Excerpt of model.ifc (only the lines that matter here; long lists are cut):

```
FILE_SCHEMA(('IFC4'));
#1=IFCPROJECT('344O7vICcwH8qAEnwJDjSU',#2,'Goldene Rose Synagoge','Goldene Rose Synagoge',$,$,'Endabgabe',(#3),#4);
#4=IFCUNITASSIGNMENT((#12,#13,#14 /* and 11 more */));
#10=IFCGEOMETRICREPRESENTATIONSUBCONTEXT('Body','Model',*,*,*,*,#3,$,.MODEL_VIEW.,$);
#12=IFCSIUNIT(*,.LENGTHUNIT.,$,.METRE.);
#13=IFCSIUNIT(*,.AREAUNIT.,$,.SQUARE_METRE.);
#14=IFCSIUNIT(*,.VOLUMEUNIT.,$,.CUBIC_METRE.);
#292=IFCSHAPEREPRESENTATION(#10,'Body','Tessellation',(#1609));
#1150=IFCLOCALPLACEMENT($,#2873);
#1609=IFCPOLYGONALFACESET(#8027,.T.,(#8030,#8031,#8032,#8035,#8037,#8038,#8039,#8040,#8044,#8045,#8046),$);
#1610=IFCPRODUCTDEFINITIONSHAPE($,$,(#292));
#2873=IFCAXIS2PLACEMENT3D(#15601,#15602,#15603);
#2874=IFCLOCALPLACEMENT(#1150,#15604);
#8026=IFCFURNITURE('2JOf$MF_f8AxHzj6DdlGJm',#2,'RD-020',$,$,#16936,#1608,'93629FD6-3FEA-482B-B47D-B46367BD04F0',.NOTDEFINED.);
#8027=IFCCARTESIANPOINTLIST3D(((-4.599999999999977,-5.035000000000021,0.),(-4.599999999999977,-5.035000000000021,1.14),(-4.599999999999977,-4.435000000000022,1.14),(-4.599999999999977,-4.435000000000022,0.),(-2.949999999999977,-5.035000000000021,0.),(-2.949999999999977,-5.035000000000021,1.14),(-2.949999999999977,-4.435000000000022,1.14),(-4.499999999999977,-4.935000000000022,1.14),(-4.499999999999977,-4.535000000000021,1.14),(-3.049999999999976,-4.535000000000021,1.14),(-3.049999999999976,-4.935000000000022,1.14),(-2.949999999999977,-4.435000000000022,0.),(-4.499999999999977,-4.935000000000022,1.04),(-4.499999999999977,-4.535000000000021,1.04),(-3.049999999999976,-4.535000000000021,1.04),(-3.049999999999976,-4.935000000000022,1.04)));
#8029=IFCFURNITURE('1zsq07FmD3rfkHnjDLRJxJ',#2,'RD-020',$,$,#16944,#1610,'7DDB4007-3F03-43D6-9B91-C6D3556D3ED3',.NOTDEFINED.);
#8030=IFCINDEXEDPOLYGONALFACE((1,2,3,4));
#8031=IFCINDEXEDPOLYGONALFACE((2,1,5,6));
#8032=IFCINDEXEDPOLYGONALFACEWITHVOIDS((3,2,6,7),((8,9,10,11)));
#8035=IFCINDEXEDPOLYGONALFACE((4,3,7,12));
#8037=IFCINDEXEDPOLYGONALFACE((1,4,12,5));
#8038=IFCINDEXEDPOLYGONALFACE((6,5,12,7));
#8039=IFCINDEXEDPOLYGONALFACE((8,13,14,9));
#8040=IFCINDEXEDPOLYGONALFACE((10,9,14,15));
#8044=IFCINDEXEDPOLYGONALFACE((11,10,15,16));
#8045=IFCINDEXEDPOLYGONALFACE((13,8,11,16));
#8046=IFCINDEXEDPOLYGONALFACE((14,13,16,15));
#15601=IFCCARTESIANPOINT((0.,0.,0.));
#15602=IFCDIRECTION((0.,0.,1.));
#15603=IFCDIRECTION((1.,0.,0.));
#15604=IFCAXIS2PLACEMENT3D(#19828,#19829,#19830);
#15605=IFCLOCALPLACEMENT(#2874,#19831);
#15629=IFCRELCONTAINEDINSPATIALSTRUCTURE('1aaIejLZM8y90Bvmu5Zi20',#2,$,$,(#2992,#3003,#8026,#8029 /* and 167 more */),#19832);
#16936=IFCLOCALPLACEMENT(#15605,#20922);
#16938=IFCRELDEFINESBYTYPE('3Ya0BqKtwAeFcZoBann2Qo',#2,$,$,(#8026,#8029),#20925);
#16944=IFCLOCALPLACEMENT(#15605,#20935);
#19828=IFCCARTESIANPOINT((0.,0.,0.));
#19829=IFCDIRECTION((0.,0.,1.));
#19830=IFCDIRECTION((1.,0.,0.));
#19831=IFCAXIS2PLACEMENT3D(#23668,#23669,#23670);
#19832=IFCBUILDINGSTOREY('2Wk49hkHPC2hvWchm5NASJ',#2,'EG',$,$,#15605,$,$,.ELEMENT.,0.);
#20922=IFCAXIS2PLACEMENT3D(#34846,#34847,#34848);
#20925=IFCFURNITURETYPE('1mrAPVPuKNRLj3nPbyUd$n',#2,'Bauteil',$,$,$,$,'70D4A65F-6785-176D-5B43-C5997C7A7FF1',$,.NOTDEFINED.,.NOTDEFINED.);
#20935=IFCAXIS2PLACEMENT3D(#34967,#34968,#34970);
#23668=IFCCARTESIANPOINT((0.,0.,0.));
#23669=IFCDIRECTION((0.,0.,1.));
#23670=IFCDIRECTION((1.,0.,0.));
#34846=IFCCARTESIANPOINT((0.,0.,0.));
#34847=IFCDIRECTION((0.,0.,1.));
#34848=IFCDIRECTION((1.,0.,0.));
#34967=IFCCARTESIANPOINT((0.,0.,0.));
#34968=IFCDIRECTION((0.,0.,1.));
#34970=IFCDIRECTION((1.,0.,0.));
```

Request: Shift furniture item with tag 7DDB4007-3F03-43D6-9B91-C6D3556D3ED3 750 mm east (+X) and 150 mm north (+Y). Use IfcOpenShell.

```python
import ifcopenshell
import ifcopenshell.api.geometry
import ifcopenshell.util.placement
import ifcopenshell.util.unit

model = ifcopenshell.open("model.ifc")
unit_scale = ifcopenshell.util.unit.calculate_unit_scale(model)

item = model.by_id(8029)
matrix = ifcopenshell.util.placement.get_local_placement(item.ObjectPlacement)
matrix[0, 3] += 0.75 / unit_scale
matrix[1, 3] += 0.15 / unit_scale
ifcopenshell.api.geometry.edit_object_placement(model, product=item, matrix=matrix, is_si=False)

print(ifcopenshell.util.placement.get_local_placement(item.ObjectPlacement).round(3) + 0.0)

model.write("model_edited.ifc")
```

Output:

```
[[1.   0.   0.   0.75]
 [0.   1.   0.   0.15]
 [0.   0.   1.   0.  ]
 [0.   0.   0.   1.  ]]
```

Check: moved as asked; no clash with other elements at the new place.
